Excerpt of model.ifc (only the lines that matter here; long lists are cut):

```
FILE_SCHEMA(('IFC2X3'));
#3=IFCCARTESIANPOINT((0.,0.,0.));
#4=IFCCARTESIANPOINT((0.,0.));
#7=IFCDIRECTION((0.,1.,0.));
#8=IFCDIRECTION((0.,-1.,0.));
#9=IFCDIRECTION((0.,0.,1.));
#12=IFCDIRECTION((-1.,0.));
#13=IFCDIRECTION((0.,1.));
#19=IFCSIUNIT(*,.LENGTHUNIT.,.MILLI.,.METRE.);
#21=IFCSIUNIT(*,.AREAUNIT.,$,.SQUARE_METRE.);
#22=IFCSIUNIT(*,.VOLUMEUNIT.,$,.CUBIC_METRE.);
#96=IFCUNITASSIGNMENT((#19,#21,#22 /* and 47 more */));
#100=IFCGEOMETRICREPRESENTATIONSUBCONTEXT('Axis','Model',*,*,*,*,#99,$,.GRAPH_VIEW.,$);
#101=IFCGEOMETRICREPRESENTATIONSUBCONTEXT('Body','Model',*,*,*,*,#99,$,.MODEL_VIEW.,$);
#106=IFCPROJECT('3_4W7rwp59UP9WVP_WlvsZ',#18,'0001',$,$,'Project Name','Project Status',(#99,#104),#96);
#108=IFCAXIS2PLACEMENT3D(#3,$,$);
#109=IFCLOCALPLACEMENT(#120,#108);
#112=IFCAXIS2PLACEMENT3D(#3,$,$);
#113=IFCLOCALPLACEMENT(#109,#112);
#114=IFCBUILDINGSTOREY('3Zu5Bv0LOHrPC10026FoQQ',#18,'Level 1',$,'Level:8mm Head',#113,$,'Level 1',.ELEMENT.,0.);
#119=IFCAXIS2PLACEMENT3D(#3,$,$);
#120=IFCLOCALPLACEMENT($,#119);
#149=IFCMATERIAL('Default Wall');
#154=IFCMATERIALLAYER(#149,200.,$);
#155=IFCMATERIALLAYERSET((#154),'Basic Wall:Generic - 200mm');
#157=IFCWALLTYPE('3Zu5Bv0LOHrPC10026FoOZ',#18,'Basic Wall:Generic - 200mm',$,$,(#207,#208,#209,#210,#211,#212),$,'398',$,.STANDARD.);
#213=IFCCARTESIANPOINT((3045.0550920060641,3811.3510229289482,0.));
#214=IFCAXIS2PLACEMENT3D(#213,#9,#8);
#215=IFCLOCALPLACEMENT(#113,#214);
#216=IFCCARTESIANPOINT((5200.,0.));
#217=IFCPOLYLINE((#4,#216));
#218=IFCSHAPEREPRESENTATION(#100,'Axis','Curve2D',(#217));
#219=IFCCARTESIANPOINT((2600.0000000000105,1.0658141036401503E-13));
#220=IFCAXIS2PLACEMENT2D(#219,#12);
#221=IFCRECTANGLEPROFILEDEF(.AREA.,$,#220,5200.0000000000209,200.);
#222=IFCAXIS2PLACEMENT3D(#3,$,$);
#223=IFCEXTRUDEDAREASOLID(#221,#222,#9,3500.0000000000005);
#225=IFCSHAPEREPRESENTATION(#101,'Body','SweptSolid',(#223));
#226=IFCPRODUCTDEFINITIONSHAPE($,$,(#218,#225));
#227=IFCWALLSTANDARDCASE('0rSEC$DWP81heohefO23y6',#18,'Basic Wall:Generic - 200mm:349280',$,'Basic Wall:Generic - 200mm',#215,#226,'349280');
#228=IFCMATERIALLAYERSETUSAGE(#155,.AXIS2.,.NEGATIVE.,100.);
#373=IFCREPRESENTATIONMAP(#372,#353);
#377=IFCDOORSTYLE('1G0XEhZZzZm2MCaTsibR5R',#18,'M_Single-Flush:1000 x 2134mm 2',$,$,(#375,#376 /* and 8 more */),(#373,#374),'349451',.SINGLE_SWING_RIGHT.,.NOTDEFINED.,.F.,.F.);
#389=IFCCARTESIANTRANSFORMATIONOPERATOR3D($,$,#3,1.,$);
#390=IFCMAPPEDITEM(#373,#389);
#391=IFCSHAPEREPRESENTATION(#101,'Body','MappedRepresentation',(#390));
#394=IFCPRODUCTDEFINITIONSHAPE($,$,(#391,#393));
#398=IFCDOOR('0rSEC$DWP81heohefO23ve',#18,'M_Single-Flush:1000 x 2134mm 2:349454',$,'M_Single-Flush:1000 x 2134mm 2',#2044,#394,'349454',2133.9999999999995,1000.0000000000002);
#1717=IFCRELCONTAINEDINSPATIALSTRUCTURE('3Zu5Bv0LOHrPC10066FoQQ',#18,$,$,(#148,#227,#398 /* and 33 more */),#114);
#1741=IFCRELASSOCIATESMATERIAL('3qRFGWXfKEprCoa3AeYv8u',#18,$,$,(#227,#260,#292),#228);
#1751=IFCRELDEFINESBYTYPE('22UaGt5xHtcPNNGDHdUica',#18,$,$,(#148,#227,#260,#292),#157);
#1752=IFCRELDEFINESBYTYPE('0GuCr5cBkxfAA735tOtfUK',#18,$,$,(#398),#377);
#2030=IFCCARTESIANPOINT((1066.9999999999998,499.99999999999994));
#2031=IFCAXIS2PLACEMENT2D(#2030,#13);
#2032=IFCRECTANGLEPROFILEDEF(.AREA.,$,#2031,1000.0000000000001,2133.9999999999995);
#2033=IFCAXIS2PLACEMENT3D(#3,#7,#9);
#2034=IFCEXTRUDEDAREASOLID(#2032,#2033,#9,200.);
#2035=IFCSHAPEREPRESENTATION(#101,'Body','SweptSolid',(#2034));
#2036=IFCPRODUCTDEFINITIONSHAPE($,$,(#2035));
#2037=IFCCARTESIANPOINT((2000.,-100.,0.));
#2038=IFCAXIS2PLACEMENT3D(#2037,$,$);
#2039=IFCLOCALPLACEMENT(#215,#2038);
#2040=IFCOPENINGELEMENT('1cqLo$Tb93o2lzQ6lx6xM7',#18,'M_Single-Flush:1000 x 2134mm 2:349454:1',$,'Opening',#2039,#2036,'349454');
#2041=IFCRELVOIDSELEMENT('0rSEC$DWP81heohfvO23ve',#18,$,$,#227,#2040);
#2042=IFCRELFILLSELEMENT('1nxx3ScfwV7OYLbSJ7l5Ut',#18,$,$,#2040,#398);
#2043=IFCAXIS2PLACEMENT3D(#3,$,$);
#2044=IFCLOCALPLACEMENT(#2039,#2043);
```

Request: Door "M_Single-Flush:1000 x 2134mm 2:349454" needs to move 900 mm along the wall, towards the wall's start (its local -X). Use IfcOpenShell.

```python
import ifcopenshell
import ifcopenshell.api.geometry
import ifcopenshell.util.placement
import ifcopenshell.util.unit

model = ifcopenshell.open("model.ifc")
unit_scale = ifcopenshell.util.unit.calculate_unit_scale(model)

door = model.by_guid("0rSEC$DWP81heohefO23ve")
opening = door.FillsVoids[0].RelatingOpeningElement
wall = opening.VoidsElements[0].RelatingBuildingElement

wall_matrix = ifcopenshell.util.placement.get_local_placement(wall.ObjectPlacement)
shift = wall_matrix[:3, 0] * -0.9 / unit_scale
before = ifcopenshell.util.placement.get_local_placement(door.ObjectPlacement)[:3, 3].copy()

# The door is placed relative to its opening, so it follows when the opening moves.
matrix = ifcopenshell.util.placement.get_local_placement(opening.ObjectPlacement)
matrix[:3, 3] += shift
ifcopenshell.api.geometry.edit_object_placement(
    model, product=opening, matrix=matrix, is_si=False, should_transform_children=True
)

after = ifcopenshell.util.placement.get_local_placement(door.ObjectPlacement)[:3, 3]
print("door moved by", (after - before).round(3) + 0.0)

model.write("model_edited.ifc")
```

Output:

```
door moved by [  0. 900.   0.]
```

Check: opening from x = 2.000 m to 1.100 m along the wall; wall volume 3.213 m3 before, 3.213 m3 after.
